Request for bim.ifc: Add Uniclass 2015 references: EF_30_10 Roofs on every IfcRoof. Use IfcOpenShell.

First a look at what the model holds.

```python
import ifcopenshell

model = ifcopenshell.open("bim.ifc")
print(model.schema)
print("classifications:", [c.Name for c in model.by_type("IfcClassification")])
for ifc_class in ("IfcDoor", "IfcRoof", "IfcStair", "IfcWall", "IfcWindow"):
    print(ifc_class, len(model.by_type(ifc_class)))
```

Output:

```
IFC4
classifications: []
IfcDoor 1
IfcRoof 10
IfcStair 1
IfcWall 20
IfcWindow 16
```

```python
import ifcopenshell
import ifcopenshell.api.classification

model = ifcopenshell.open("bim.ifc")

system = ifcopenshell.api.classification.add_classification(model, classification="Uniclass 2015")

codes = {
    "IfcRoof": ("EF_30_10", "Roofs"),
}
for ifc_class, (code, name) in codes.items():
    products = model.by_type(ifc_class)
    ifcopenshell.api.classification.add_reference(
        model, products=products, classification=system, identification=code, name=name
    )
    print(code, len(products))

model.write("bim_updated.ifc")
```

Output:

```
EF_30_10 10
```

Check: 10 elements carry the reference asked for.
